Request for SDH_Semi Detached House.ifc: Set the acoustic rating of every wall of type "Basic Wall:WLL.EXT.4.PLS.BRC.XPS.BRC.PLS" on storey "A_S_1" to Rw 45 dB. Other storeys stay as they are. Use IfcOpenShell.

First a look at what the model holds.

```python
import ifcopenshell
import ifcopenshell.util.element

model = ifcopenshell.open("SDH_Semi Detached House.ifc")
print(model.schema)
storey = next(s for s in model.by_type("IfcBuildingStorey") if s.Name == "A_S_1")
walls = [e for e in ifcopenshell.util.element.get_decomposition(storey) if e.is_a("IfcWall")]
seen = {}
for e in walls:
    element_type = ifcopenshell.util.element.get_type(e)
    key = (element_type.Name if element_type != e and element_type else None, ifcopenshell.util.element.get_pset(e, "Pset_WallCommon", "AcousticRating"))
    seen[key] = seen.get(key, 0) + 1
for (name, value), count in sorted(seen.items(), key=str):
    print(count, "x", name, "|", value)
```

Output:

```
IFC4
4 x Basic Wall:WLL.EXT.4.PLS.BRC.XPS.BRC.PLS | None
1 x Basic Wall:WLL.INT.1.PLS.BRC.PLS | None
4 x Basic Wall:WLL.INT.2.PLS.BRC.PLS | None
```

```python
import ifcopenshell
import ifcopenshell.api.pset
import ifcopenshell.util.element

model = ifcopenshell.open("SDH_Semi Detached House.ifc")

storey = next(s for s in model.by_type("IfcBuildingStorey") if s.Name == "A_S_1")
walls = [e for e in ifcopenshell.util.element.get_decomposition(storey) if e.is_a("IfcWall")]

count = 0
for e in walls:
    element_type = ifcopenshell.util.element.get_type(e)
    if element_type in (None, e) or element_type.Name != "Basic Wall:WLL.EXT.4.PLS.BRC.XPS.BRC.PLS":
        continue
    # add_pset returns the element's existing set when there is one.
    pset = ifcopenshell.api.pset.add_pset(model, product=e, name="Pset_WallCommon")
    ifcopenshell.api.pset.edit_pset(model, pset=pset, properties={"AcousticRating": "Rw 45 dB"})
    count += 1

print(count, "walls updated")

model.write("SDH_Semi Detached House_updated.ifc")
```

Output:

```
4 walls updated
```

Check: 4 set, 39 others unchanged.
